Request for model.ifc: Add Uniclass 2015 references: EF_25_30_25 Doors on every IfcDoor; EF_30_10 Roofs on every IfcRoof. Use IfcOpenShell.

First a look at what the model holds.

```python
import ifcopenshell

model = ifcopenshell.open("model.ifc")
print(model.schema)
print("classifications:", [c.Name for c in model.by_type("IfcClassification")])
for ifc_class in ("IfcDoor", "IfcRoof", "IfcStair", "IfcWall", "IfcWindow"):
    print(ifc_class, len(model.by_type(ifc_class)))
```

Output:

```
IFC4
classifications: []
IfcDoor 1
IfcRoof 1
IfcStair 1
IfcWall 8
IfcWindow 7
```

```python
import ifcopenshell
import ifcopenshell.api.classification

model = ifcopenshell.open("model.ifc")

system = ifcopenshell.api.classification.add_classification(model, classification="Uniclass 2015")

codes = {
    "IfcDoor": ("EF_25_30_25", "Doors"),
    "IfcRoof": ("EF_30_10", "Roofs"),
}
for ifc_class, (code, name) in codes.items():
    products = model.by_type(ifc_class)
    ifcopenshell.api.classification.add_reference(
        model, products=products, classification=system, identification=code, name=name
    )
    print(code, len(products))

model.write("model_updated.ifc")
```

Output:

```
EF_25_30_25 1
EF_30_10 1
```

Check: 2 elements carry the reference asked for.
